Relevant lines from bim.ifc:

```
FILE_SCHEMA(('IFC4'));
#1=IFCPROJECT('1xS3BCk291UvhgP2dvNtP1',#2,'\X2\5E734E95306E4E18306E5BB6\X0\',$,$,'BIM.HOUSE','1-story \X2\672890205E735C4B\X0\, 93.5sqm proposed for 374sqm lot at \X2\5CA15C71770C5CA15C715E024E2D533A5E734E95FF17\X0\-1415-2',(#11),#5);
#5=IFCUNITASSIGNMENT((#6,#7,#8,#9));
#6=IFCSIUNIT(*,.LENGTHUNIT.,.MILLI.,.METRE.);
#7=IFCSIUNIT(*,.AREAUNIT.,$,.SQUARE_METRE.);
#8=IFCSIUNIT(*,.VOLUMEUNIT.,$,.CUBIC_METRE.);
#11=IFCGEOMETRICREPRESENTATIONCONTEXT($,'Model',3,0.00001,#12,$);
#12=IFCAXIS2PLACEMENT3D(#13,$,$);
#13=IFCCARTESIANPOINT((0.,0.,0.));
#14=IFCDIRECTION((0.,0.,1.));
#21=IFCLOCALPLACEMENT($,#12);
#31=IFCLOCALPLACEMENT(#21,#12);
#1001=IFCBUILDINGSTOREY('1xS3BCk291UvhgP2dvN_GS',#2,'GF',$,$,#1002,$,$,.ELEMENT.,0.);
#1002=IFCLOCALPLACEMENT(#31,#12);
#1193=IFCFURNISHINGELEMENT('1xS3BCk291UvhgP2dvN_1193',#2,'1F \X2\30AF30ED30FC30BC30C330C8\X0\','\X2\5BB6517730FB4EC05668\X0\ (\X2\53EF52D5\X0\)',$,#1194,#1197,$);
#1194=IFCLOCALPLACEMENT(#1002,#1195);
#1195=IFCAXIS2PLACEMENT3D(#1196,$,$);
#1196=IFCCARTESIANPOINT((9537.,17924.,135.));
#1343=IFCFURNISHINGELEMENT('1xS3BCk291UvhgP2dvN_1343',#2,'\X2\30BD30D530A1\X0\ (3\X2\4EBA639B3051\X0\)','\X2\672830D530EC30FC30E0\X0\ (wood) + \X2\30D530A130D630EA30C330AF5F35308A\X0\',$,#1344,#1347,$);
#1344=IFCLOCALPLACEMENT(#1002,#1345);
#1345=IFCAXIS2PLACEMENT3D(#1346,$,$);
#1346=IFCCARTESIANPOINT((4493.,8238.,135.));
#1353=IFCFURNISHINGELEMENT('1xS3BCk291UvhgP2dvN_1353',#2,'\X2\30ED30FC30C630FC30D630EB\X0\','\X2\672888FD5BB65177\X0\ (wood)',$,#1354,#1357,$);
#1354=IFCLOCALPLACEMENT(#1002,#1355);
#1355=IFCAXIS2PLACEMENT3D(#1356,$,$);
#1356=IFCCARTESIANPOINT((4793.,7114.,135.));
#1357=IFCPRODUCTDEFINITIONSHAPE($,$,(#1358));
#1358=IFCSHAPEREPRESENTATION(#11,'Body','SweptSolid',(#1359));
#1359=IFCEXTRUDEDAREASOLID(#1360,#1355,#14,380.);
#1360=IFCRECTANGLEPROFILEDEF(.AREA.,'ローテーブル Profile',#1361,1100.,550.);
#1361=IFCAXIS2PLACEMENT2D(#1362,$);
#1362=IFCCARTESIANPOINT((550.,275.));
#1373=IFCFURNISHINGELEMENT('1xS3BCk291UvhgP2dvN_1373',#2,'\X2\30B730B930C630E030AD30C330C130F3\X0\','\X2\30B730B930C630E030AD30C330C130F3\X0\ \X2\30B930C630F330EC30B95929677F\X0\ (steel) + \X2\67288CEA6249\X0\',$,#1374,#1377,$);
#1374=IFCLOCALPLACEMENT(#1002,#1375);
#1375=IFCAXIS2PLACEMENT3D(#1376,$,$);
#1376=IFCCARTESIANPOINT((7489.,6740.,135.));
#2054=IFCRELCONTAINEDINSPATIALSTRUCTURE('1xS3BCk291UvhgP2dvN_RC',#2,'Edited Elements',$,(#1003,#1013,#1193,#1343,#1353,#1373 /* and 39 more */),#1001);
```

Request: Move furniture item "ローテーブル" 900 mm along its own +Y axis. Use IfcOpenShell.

```python
import ifcopenshell
import ifcopenshell.api.geometry
import ifcopenshell.util.placement
import ifcopenshell.util.unit

model = ifcopenshell.open("bim.ifc")
unit_scale = ifcopenshell.util.unit.calculate_unit_scale(model)

item = model.by_guid("1xS3BCk291UvhgP2dvN_1353")
matrix = ifcopenshell.util.placement.get_local_placement(item.ObjectPlacement)
matrix[:3, 3] += matrix[:3, 1] * 0.9 / unit_scale
ifcopenshell.api.geometry.edit_object_placement(model, product=item, matrix=matrix, is_si=False)

print(ifcopenshell.util.placement.get_local_placement(item.ObjectPlacement).round(3) + 0.0)

model.write("bim_v2.ifc")
```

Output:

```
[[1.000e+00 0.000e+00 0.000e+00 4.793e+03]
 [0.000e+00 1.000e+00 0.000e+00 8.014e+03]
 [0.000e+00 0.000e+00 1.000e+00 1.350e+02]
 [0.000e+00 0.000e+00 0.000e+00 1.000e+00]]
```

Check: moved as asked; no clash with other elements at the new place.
